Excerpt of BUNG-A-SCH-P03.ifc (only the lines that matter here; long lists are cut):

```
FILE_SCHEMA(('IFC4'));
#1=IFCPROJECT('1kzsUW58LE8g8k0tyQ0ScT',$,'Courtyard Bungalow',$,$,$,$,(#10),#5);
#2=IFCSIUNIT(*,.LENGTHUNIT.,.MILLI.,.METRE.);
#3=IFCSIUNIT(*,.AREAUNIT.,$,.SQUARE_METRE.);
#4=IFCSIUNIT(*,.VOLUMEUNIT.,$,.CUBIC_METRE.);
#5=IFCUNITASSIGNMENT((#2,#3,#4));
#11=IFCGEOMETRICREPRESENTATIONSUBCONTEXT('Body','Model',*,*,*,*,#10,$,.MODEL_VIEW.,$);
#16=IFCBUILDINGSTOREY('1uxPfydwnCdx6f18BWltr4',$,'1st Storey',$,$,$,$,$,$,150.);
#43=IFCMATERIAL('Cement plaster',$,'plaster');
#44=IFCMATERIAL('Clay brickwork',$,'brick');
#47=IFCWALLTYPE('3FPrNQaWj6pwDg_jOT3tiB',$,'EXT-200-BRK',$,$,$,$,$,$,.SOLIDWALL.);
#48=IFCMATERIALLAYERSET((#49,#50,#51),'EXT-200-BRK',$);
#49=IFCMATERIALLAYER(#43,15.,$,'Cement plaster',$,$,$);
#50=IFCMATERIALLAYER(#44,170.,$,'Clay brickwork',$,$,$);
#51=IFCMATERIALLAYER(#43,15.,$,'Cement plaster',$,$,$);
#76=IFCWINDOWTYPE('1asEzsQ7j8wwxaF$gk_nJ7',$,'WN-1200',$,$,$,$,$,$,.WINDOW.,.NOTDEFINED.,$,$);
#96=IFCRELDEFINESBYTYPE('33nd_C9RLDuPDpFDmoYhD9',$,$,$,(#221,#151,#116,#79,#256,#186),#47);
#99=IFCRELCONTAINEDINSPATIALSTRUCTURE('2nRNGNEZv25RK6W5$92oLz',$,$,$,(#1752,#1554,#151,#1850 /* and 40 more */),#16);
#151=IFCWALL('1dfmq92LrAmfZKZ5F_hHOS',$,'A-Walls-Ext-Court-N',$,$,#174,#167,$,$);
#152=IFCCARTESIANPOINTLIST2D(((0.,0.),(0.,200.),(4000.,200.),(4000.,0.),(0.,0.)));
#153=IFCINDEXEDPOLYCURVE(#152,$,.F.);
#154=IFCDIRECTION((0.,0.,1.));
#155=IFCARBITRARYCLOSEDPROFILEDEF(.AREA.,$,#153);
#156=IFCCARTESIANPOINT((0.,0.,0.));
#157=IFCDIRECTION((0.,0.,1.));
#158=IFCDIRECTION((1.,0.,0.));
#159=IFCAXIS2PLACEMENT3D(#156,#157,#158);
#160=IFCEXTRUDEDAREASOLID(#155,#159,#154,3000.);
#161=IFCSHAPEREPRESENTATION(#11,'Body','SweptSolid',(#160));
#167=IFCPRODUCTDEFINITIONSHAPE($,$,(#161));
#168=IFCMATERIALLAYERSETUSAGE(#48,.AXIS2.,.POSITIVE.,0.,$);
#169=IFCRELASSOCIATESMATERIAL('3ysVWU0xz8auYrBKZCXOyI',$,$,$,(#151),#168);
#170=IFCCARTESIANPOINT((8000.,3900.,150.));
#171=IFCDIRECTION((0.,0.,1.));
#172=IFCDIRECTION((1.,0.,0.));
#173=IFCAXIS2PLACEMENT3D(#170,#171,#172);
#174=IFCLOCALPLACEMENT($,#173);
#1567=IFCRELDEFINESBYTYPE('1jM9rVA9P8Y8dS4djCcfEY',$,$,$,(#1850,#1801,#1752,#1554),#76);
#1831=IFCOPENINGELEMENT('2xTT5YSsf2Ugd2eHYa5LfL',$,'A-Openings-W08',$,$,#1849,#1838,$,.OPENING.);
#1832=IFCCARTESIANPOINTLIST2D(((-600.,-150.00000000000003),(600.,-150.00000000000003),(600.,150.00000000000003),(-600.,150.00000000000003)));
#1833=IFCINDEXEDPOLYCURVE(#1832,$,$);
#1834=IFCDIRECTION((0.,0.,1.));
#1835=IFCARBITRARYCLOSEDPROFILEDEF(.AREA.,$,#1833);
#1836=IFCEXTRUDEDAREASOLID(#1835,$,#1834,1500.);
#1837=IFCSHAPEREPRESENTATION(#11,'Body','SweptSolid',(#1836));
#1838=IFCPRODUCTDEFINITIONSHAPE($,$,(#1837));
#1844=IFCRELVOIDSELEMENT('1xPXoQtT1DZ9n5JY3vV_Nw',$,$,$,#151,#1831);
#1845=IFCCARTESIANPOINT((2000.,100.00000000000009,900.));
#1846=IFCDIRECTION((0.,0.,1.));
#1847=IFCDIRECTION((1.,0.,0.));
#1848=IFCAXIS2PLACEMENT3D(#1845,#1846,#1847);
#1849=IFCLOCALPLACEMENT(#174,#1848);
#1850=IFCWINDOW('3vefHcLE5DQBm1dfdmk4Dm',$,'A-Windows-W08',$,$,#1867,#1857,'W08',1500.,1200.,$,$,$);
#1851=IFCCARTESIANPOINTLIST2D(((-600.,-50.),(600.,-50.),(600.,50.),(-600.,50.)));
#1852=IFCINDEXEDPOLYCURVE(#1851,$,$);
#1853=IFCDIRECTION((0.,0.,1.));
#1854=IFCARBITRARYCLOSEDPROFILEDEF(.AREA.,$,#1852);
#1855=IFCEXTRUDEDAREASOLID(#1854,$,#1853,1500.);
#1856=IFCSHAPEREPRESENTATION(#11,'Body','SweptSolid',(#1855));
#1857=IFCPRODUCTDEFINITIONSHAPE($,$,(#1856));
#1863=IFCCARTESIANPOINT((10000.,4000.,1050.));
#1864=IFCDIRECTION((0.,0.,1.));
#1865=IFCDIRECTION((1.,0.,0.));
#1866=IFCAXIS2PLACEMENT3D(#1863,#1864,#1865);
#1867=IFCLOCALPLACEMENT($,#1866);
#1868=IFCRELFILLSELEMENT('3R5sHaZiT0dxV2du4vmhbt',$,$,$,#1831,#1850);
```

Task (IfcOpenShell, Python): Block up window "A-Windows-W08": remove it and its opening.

```python
import ifcopenshell
import ifcopenshell.api.feature
import ifcopenshell.api.root
import ifcopenshell.geom
import ifcopenshell.util.shape

model = ifcopenshell.open("BUNG-A-SCH-P03.ifc")
settings = ifcopenshell.geom.settings()


def volume(element):
    """Net volume in cubic metres, openings subtracted."""
    shape = ifcopenshell.geom.create_shape(settings, element)
    return ifcopenshell.util.shape.get_volume(shape.geometry)


window = model.by_guid("3vefHcLE5DQBm1dfdmk4Dm")
opening = window.FillsVoids[0].RelatingOpeningElement
wall = opening.VoidsElements[0].RelatingBuildingElement
before = volume(wall)

ifcopenshell.api.root.remove_product(model, product=window)
ifcopenshell.api.feature.remove_feature(model, feature=opening)

after = volume(wall)

print(f"wall volume {before:.3f} -> {after:.3f} m3")

model.write("BUNG-A-SCH-P03_v2.ifc")
```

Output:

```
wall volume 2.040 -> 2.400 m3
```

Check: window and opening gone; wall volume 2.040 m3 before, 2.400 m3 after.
